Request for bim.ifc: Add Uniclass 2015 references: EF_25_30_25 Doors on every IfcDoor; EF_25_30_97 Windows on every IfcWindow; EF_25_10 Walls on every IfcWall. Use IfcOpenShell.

First a look at what the model holds.

```python
import ifcopenshell

model = ifcopenshell.open("bim.ifc")
print(model.schema)
print("classifications:", [c.Name for c in model.by_type("IfcClassification")])
for ifc_class in ("IfcDoor", "IfcRoof", "IfcStair", "IfcWall", "IfcWindow"):
    print(ifc_class, len(model.by_type(ifc_class)))
```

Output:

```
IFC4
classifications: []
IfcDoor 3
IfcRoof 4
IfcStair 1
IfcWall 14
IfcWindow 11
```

```python
import ifcopenshell
import ifcopenshell.api.classification

model = ifcopenshell.open("bim.ifc")

system = ifcopenshell.api.classification.add_classification(model, classification="Uniclass 2015")

codes = {
    "IfcDoor": ("EF_25_30_25", "Doors"),
    "IfcWindow": ("EF_25_30_97", "Windows"),
    "IfcWall": ("EF_25_10", "Walls"),
}
for ifc_class, (code, name) in codes.items():
    products = model.by_type(ifc_class)
    ifcopenshell.api.classification.add_reference(
        model, products=products, classification=system, identification=code, name=name
    )
    print(code, len(products))

model.write("bim_v2.ifc")
```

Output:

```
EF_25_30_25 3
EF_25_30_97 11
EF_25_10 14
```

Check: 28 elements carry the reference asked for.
